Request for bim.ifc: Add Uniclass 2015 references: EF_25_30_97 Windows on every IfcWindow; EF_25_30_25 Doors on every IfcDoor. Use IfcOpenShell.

First a look at what the model holds.

```python
import ifcopenshell

model = ifcopenshell.open("bim.ifc")
print(model.schema)
print("classifications:", [c.Name for c in model.by_type("IfcClassification")])
for ifc_class in ("IfcDoor", "IfcRoof", "IfcStair", "IfcWall", "IfcWindow"):
    print(ifc_class, len(model.by_type(ifc_class)))
```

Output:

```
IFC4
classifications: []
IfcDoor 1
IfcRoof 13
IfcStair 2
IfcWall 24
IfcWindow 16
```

```python
import ifcopenshell
import ifcopenshell.api.classification

model = ifcopenshell.open("bim.ifc")

system = ifcopenshell.api.classification.add_classification(model, classification="Uniclass 2015")

codes = {
    "IfcWindow": ("EF_25_30_97", "Windows"),
    "IfcDoor": ("EF_25_30_25", "Doors"),
}
for ifc_class, (code, name) in codes.items():
    products = model.by_type(ifc_class)
    ifcopenshell.api.classification.add_reference(
        model, products=products, classification=system, identification=code, name=name
    )
    print(code, len(products))

model.write("bim_edited.ifc")
```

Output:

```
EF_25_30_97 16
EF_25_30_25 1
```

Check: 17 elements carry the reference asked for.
